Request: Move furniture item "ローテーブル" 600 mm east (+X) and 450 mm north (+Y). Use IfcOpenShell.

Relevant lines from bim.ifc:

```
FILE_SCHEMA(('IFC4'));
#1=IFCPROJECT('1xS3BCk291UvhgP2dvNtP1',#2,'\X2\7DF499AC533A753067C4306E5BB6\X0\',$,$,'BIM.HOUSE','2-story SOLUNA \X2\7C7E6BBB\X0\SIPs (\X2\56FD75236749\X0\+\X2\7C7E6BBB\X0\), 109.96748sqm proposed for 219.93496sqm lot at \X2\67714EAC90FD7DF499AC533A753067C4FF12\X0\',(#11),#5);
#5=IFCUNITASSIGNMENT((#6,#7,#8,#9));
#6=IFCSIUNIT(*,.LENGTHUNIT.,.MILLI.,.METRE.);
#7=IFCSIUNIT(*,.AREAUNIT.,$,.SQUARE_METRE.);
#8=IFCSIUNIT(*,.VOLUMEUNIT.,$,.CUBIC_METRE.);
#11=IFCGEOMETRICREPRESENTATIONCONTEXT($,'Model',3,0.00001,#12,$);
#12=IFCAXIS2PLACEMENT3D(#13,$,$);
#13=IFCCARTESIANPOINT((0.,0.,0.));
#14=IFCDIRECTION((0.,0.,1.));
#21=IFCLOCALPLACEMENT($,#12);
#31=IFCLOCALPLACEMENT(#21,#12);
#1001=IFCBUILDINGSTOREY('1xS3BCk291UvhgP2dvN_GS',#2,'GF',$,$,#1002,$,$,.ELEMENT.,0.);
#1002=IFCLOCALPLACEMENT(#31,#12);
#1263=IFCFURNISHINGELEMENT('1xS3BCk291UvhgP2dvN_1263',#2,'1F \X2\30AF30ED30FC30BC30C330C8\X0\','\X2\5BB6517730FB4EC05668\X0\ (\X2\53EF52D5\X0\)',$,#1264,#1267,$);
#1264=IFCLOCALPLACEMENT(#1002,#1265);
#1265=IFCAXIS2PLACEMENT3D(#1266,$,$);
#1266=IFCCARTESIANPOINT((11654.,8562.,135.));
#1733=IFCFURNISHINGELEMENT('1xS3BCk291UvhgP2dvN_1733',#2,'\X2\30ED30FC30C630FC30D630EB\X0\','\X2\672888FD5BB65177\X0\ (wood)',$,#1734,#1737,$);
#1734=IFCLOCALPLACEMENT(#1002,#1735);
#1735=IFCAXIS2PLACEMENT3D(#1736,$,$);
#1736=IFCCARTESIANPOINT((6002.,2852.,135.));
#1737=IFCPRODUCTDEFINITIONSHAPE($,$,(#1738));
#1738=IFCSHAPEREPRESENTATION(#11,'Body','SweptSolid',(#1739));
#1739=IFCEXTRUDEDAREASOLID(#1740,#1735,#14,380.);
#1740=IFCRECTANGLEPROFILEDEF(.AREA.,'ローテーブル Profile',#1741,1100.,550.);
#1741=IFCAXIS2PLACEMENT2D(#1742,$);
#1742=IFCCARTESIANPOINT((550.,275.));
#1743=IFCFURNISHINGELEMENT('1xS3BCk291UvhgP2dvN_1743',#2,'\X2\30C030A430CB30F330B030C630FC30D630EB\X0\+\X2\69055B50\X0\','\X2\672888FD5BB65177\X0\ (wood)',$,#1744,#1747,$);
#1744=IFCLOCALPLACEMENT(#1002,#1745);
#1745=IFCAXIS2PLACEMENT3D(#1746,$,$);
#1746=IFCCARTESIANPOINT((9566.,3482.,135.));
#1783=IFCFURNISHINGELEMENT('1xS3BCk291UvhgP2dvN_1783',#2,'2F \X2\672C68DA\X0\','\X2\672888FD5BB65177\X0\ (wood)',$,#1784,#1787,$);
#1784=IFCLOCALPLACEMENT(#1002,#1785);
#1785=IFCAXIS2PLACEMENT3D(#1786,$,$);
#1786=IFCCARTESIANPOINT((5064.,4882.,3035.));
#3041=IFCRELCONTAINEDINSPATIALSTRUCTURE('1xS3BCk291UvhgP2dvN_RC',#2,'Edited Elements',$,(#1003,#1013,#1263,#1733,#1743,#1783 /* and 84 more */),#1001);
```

```python
import ifcopenshell
import ifcopenshell.api.geometry
import ifcopenshell.util.placement
import ifcopenshell.util.unit

model = ifcopenshell.open("bim.ifc")
unit_scale = ifcopenshell.util.unit.calculate_unit_scale(model)

item = model.by_id(1733)
matrix = ifcopenshell.util.placement.get_local_placement(item.ObjectPlacement)
matrix[0, 3] += 0.6 / unit_scale
matrix[1, 3] += 0.45 / unit_scale
ifcopenshell.api.geometry.edit_object_placement(model, product=item, matrix=matrix, is_si=False)

print(ifcopenshell.util.placement.get_local_placement(item.ObjectPlacement).round(3) + 0.0)

model.write("bim_updated.ifc")
```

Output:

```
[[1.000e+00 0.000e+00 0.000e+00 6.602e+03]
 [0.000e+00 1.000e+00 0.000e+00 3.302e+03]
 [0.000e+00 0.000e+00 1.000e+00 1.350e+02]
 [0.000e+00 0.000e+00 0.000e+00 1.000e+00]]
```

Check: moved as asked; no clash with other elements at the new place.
